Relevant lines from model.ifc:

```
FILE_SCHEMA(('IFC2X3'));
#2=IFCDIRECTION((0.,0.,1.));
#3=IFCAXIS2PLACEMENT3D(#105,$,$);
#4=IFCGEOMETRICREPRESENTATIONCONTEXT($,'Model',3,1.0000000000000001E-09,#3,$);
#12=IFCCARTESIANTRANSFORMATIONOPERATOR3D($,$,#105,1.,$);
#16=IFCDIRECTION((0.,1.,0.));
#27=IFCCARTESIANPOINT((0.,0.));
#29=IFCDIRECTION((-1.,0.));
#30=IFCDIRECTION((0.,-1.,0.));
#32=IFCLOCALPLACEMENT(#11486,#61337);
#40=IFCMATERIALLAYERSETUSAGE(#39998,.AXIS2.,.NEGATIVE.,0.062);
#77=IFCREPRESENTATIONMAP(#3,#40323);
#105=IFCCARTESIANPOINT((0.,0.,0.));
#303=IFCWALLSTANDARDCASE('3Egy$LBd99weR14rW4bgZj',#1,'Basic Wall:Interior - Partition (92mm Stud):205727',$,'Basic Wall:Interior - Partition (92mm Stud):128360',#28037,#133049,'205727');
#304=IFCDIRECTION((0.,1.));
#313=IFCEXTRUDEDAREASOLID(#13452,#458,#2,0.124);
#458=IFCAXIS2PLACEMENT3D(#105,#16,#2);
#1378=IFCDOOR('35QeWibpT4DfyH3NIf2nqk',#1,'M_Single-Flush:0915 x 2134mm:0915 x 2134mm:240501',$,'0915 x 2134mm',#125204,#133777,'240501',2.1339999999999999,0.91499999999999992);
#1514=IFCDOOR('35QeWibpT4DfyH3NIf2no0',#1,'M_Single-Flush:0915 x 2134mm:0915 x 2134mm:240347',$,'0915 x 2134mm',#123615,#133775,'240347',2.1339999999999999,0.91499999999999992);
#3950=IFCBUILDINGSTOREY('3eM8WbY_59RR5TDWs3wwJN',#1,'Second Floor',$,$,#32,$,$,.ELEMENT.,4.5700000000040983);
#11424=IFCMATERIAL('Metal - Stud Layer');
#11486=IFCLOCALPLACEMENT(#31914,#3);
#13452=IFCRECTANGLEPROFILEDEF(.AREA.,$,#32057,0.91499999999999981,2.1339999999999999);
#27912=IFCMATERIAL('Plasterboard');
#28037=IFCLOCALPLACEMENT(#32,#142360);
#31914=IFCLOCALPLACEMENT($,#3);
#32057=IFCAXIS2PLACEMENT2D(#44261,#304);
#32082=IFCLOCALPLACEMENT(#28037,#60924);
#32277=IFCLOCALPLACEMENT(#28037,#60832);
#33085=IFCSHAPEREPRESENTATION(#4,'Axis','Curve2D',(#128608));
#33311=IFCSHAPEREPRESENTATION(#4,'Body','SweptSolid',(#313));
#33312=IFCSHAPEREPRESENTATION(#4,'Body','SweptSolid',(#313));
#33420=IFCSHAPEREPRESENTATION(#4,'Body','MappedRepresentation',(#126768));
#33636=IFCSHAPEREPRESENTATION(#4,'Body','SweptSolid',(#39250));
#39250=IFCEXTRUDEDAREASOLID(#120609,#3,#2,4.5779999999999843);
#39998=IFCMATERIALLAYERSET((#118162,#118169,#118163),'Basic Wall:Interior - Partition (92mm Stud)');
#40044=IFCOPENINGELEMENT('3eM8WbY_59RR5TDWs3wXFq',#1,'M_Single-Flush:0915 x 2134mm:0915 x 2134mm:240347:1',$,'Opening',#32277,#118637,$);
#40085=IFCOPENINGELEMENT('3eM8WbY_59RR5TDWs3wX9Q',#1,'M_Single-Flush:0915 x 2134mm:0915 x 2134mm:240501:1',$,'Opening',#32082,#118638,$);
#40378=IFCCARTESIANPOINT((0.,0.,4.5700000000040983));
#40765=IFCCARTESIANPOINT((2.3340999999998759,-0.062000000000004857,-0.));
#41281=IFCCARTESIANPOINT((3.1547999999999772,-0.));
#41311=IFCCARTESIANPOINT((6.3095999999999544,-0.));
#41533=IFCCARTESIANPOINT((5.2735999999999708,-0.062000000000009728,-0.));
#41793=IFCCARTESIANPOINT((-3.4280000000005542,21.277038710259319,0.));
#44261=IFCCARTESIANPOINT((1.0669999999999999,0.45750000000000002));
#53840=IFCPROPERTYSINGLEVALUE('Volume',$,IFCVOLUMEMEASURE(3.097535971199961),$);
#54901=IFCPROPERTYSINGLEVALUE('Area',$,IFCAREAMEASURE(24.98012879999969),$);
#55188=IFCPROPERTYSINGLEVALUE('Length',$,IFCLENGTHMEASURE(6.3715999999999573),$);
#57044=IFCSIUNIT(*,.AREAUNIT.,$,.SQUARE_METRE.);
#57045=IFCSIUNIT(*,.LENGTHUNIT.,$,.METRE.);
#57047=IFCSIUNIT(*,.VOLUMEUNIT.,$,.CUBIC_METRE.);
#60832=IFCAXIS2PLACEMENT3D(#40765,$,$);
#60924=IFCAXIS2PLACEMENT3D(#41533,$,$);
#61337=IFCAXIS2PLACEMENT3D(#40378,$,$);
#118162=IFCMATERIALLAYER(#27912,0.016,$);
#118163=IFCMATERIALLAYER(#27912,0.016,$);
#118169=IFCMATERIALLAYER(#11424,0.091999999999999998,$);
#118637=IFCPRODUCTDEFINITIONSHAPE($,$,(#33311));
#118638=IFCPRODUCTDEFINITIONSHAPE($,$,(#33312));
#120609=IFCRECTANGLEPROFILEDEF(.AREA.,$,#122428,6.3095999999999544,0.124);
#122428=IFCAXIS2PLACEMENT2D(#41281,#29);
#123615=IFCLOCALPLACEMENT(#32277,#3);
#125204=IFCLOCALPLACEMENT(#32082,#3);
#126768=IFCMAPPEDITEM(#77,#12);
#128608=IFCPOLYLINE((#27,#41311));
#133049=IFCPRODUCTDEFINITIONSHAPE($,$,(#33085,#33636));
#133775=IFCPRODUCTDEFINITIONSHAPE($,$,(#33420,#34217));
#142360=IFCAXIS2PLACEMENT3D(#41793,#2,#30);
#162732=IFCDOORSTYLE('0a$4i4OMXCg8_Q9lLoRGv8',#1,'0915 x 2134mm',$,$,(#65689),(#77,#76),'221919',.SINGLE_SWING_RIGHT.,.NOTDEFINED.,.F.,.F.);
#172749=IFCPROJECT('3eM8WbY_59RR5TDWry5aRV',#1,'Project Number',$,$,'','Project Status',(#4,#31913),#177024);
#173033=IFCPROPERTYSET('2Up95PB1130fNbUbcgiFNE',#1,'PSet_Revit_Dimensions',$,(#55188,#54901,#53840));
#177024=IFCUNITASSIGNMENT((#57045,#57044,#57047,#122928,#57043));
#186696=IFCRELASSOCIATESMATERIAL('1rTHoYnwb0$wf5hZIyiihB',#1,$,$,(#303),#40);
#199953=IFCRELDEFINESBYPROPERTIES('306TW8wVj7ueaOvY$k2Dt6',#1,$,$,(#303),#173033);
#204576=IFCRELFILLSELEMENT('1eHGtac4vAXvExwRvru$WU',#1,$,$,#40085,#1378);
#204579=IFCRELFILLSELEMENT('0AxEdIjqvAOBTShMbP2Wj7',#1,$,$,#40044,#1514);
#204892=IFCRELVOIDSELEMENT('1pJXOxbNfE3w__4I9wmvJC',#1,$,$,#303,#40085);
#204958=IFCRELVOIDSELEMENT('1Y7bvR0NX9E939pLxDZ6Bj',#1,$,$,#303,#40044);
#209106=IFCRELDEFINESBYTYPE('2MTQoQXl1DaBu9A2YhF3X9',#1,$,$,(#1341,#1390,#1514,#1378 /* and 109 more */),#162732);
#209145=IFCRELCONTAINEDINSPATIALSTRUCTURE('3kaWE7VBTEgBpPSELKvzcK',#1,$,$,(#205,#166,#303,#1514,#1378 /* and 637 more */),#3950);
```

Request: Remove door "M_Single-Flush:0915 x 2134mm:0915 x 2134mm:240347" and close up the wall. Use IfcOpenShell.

```python
import ifcopenshell
import ifcopenshell.api.feature
import ifcopenshell.api.pset
import ifcopenshell.api.root
import ifcopenshell.geom
import ifcopenshell.util.element
import ifcopenshell.util.shape
import ifcopenshell.util.unit

model = ifcopenshell.open("model.ifc")
area_scale = ifcopenshell.util.unit.calculate_unit_scale(model, "AREAUNIT")
volume_scale = ifcopenshell.util.unit.calculate_unit_scale(model, "VOLUMEUNIT")
settings = ifcopenshell.geom.settings()


def volume(element):
    """Net volume in cubic metres, openings subtracted."""
    shape = ifcopenshell.geom.create_shape(settings, element)
    return ifcopenshell.util.shape.get_volume(shape.geometry)


door = model.by_id(1514)
opening = door.FillsVoids[0].RelatingOpeningElement
wall = opening.VoidsElements[0].RelatingBuildingElement
before = volume(wall)

ifcopenshell.api.root.remove_product(model, product=door)
ifcopenshell.api.feature.remove_feature(model, feature=opening)

after = volume(wall)
thickness = 0.124  # wall thickness in metres

# Update the wall's stored quantities.
pset = model.by_id(ifcopenshell.util.element.get_pset(wall, "PSet_Revit_Dimensions", should_inherit=False)["id"])
ifcopenshell.api.pset.edit_pset(model, pset=pset, properties={
    "Area": model.create_entity("IfcAreaMeasure", after / thickness / area_scale),
    "Volume": model.create_entity("IfcVolumeMeasure", after / volume_scale),
})

print(f"wall volume {before:.3f} -> {after:.3f} m3")

model.write("model_updated.ifc")
```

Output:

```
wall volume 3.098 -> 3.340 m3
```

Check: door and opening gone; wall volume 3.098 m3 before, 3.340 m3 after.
